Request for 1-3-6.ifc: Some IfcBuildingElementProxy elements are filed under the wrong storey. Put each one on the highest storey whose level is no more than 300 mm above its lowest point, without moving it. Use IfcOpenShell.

First a look at what the model holds.

```python
import ifcopenshell
import ifcopenshell.util.element
import ifcopenshell.util.placement

model = ifcopenshell.open("1-3-6.ifc")
print(model.schema)
for storey in model.by_type("IfcBuildingStorey"):
    level = ifcopenshell.util.placement.get_storey_elevation(storey)
    count = sum(e.is_a("IfcBuildingElementProxy") for e in ifcopenshell.util.element.get_contained(storey))
    print(storey.id(), storey.Name, round(level, 3), count, sep=" | ")
```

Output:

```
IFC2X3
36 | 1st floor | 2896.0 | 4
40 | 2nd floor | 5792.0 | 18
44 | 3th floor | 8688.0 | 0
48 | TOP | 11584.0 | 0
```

```python
import ifcopenshell
import ifcopenshell.api.spatial
import ifcopenshell.geom
import ifcopenshell.util.element
import ifcopenshell.util.placement
import ifcopenshell.util.shape
import ifcopenshell.util.unit

model = ifcopenshell.open("1-3-6.ifc")
unit_scale = ifcopenshell.util.unit.calculate_unit_scale(model)
settings = ifcopenshell.geom.settings()

levels = sorted(
    ((ifcopenshell.util.placement.get_storey_elevation(s) * unit_scale, s) for s in model.by_type("IfcBuildingStorey")),
    key=lambda pair: pair[0],
)

for e in model.by_type("IfcBuildingElementProxy"):
    current = e.ContainedInStructure[0].RelatingStructure if e.ContainedInStructure else None
    if current is None or not current.is_a("IfcBuildingStorey"):
        continue
    shape = ifcopenshell.geom.create_shape(settings, e)
    bottom = ifcopenshell.util.shape.get_shape_bottom_elevation(shape, shape.geometry)
    below = [s for level, s in levels if level <= bottom + 0.3]
    storey = below[-1] if below else levels[0][1]
    if storey != current:
        # assign_container keeps the world position.
        ifcopenshell.api.spatial.assign_container(model, products=[e], relating_structure=storey)
        print(e.id(), current.Name, "->", storey.Name)

model.write("1-3-6-out.ifc")
```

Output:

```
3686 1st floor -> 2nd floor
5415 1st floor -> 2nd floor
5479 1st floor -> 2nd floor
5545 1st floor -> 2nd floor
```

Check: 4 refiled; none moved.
